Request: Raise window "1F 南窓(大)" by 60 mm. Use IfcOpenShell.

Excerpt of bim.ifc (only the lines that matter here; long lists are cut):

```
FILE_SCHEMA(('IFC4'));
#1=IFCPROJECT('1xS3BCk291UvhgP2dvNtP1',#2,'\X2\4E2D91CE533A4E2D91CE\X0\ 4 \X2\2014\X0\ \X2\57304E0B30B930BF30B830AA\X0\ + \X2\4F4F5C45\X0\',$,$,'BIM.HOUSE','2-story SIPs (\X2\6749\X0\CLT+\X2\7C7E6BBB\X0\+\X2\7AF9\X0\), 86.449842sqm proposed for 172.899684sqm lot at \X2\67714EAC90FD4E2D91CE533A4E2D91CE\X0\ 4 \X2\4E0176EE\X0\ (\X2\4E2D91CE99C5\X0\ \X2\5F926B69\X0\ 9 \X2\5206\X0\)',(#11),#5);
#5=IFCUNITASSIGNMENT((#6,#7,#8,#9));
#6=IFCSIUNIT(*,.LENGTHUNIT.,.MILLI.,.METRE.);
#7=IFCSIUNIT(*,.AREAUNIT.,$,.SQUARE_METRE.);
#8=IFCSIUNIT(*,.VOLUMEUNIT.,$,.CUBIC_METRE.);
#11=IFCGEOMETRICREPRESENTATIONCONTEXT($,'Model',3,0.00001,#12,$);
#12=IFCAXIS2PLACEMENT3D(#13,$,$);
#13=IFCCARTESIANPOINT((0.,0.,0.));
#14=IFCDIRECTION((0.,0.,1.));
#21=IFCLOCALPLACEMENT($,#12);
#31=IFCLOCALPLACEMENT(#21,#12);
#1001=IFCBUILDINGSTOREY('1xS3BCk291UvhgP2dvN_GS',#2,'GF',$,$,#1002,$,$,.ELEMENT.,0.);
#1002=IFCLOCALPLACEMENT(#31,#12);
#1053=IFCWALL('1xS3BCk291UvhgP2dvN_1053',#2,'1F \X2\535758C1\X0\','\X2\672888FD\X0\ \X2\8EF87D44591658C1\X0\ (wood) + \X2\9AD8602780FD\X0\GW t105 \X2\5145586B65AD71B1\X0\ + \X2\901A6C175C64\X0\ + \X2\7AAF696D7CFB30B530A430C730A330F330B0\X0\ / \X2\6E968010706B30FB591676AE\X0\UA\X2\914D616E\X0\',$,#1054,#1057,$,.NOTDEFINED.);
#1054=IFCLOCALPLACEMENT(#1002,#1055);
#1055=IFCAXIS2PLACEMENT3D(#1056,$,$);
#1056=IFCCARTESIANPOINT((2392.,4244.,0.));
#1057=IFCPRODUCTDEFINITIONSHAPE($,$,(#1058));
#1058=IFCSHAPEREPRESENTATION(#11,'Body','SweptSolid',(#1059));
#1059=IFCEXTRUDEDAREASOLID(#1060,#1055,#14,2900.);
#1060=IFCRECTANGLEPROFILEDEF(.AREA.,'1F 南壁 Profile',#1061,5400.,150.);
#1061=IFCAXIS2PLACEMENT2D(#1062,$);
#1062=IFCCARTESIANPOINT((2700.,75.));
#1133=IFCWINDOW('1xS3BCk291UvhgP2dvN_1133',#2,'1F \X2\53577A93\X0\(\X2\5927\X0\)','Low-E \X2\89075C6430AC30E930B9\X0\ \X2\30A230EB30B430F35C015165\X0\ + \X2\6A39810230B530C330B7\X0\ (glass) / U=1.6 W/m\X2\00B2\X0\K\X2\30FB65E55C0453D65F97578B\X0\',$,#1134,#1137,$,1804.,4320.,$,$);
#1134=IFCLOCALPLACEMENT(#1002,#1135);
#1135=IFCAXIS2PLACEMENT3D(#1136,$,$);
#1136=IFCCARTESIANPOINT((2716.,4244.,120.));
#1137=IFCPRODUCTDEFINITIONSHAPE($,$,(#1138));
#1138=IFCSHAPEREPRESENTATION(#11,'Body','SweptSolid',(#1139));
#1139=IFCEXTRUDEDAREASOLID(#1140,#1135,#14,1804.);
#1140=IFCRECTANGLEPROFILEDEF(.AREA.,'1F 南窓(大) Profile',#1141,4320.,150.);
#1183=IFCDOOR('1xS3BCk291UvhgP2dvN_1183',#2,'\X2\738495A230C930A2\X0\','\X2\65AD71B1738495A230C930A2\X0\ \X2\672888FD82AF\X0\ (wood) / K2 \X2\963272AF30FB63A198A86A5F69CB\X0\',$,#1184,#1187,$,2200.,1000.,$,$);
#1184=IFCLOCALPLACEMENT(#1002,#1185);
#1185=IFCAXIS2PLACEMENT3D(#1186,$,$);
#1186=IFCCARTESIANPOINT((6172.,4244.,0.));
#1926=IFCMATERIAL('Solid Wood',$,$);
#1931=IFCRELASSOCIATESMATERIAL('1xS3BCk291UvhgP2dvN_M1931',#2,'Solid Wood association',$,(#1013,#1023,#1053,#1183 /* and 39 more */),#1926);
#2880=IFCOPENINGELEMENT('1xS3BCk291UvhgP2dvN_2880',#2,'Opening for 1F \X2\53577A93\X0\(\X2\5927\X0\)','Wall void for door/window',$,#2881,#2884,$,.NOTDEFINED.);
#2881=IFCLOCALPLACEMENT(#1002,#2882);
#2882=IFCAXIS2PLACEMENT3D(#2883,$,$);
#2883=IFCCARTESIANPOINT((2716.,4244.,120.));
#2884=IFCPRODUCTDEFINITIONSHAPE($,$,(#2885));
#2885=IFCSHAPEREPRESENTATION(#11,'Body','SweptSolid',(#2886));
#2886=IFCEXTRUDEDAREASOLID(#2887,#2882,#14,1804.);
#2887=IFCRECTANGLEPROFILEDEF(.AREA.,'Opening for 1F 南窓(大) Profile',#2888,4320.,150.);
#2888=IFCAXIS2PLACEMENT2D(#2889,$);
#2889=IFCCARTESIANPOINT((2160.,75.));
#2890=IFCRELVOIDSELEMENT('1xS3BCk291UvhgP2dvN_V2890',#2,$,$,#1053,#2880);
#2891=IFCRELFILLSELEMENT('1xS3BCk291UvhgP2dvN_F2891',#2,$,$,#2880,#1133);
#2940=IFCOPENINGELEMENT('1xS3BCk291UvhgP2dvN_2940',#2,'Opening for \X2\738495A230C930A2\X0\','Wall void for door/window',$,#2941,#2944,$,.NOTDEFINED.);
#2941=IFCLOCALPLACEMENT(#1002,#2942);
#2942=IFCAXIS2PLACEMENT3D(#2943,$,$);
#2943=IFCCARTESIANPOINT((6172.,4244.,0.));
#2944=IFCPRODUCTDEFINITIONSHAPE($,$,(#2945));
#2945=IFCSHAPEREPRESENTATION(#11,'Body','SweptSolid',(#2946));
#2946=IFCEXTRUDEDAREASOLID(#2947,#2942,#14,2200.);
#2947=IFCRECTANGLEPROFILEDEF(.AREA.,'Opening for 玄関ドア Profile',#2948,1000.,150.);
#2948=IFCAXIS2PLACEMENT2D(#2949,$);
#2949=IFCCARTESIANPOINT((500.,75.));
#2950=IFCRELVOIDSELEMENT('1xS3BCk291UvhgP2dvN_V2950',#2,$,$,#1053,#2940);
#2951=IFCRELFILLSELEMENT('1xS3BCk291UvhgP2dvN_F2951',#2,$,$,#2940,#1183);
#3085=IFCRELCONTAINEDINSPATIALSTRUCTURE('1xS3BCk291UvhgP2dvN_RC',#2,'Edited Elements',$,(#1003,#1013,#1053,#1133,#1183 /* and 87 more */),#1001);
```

```python
import numpy as np
import ifcopenshell
import ifcopenshell.api.geometry
import ifcopenshell.util.placement
import ifcopenshell.util.unit

model = ifcopenshell.open("bim.ifc")
unit_scale = ifcopenshell.util.unit.calculate_unit_scale(model)

window = model.by_guid("1xS3BCk291UvhgP2dvN_1133")
opening = window.FillsVoids[0].RelatingOpeningElement
dz = 0.06 / unit_scale

shift = np.array([0.0, 0.0, dz])
# The window is not placed relative to its opening, so move both.
for product in (opening, window):
    matrix = ifcopenshell.util.placement.get_local_placement(product.ObjectPlacement)
    matrix[:3, 3] += shift
    ifcopenshell.api.geometry.edit_object_placement(model, product=product, matrix=matrix, is_si=False)

print(f"moved by {dz * unit_scale:+.3f} m")

model.write("bim_v2.ifc")
```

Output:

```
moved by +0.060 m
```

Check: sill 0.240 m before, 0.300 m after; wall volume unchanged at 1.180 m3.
